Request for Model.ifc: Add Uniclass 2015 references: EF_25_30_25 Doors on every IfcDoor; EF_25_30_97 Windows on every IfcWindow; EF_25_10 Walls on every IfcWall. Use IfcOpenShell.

First a look at what the model holds.

```python
import ifcopenshell

model = ifcopenshell.open("Model.ifc")
print(model.schema)
print("classifications:", [c.Name for c in model.by_type("IfcClassification")])
for ifc_class in ("IfcDoor", "IfcRoof", "IfcStair", "IfcWall", "IfcWindow"):
    print(ifc_class, len(model.by_type(ifc_class)))
```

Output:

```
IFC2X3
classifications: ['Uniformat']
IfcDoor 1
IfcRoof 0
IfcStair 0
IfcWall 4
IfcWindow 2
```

```python
import ifcopenshell
import ifcopenshell.api.classification

model = ifcopenshell.open("Model.ifc")

# IFC2X3 requires Source and Edition and has no link from the project to the system.
system = model.create_entity("IfcClassification", Source="NBS", Edition="2015", Name="Uniclass 2015")

codes = {
    "IfcDoor": ("EF_25_30_25", "Doors"),
    "IfcWindow": ("EF_25_30_97", "Windows"),
    "IfcWall": ("EF_25_10", "Walls"),
}
for ifc_class, (code, name) in codes.items():
    products = model.by_type(ifc_class)
    ifcopenshell.api.classification.add_reference(
        model, products=products, classification=system, identification=code, name=name
    )
    print(code, len(products))

model.write("Model_edited.ifc")
```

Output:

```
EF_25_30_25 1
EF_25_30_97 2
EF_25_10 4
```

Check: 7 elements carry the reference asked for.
